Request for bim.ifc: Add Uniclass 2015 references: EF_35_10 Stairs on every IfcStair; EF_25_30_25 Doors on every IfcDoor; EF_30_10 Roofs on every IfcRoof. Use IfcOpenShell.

First a look at what the model holds.

```python
import ifcopenshell

model = ifcopenshell.open("bim.ifc")
print(model.schema)
print("classifications:", [c.Name for c in model.by_type("IfcClassification")])
for ifc_class in ("IfcDoor", "IfcRoof", "IfcStair", "IfcWall", "IfcWindow"):
    print(ifc_class, len(model.by_type(ifc_class)))
```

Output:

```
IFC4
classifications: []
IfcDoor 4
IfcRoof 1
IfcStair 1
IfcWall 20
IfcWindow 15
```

```python
import ifcopenshell
import ifcopenshell.api.classification

model = ifcopenshell.open("bim.ifc")

system = ifcopenshell.api.classification.add_classification(model, classification="Uniclass 2015")

codes = {
    "IfcStair": ("EF_35_10", "Stairs"),
    "IfcDoor": ("EF_25_30_25", "Doors"),
    "IfcRoof": ("EF_30_10", "Roofs"),
}
for ifc_class, (code, name) in codes.items():
    products = model.by_type(ifc_class)
    ifcopenshell.api.classification.add_reference(
        model, products=products, classification=system, identification=code, name=name
    )
    print(code, len(products))

model.write("bim_edited.ifc")
```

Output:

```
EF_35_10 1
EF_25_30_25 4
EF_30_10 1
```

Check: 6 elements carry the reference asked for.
